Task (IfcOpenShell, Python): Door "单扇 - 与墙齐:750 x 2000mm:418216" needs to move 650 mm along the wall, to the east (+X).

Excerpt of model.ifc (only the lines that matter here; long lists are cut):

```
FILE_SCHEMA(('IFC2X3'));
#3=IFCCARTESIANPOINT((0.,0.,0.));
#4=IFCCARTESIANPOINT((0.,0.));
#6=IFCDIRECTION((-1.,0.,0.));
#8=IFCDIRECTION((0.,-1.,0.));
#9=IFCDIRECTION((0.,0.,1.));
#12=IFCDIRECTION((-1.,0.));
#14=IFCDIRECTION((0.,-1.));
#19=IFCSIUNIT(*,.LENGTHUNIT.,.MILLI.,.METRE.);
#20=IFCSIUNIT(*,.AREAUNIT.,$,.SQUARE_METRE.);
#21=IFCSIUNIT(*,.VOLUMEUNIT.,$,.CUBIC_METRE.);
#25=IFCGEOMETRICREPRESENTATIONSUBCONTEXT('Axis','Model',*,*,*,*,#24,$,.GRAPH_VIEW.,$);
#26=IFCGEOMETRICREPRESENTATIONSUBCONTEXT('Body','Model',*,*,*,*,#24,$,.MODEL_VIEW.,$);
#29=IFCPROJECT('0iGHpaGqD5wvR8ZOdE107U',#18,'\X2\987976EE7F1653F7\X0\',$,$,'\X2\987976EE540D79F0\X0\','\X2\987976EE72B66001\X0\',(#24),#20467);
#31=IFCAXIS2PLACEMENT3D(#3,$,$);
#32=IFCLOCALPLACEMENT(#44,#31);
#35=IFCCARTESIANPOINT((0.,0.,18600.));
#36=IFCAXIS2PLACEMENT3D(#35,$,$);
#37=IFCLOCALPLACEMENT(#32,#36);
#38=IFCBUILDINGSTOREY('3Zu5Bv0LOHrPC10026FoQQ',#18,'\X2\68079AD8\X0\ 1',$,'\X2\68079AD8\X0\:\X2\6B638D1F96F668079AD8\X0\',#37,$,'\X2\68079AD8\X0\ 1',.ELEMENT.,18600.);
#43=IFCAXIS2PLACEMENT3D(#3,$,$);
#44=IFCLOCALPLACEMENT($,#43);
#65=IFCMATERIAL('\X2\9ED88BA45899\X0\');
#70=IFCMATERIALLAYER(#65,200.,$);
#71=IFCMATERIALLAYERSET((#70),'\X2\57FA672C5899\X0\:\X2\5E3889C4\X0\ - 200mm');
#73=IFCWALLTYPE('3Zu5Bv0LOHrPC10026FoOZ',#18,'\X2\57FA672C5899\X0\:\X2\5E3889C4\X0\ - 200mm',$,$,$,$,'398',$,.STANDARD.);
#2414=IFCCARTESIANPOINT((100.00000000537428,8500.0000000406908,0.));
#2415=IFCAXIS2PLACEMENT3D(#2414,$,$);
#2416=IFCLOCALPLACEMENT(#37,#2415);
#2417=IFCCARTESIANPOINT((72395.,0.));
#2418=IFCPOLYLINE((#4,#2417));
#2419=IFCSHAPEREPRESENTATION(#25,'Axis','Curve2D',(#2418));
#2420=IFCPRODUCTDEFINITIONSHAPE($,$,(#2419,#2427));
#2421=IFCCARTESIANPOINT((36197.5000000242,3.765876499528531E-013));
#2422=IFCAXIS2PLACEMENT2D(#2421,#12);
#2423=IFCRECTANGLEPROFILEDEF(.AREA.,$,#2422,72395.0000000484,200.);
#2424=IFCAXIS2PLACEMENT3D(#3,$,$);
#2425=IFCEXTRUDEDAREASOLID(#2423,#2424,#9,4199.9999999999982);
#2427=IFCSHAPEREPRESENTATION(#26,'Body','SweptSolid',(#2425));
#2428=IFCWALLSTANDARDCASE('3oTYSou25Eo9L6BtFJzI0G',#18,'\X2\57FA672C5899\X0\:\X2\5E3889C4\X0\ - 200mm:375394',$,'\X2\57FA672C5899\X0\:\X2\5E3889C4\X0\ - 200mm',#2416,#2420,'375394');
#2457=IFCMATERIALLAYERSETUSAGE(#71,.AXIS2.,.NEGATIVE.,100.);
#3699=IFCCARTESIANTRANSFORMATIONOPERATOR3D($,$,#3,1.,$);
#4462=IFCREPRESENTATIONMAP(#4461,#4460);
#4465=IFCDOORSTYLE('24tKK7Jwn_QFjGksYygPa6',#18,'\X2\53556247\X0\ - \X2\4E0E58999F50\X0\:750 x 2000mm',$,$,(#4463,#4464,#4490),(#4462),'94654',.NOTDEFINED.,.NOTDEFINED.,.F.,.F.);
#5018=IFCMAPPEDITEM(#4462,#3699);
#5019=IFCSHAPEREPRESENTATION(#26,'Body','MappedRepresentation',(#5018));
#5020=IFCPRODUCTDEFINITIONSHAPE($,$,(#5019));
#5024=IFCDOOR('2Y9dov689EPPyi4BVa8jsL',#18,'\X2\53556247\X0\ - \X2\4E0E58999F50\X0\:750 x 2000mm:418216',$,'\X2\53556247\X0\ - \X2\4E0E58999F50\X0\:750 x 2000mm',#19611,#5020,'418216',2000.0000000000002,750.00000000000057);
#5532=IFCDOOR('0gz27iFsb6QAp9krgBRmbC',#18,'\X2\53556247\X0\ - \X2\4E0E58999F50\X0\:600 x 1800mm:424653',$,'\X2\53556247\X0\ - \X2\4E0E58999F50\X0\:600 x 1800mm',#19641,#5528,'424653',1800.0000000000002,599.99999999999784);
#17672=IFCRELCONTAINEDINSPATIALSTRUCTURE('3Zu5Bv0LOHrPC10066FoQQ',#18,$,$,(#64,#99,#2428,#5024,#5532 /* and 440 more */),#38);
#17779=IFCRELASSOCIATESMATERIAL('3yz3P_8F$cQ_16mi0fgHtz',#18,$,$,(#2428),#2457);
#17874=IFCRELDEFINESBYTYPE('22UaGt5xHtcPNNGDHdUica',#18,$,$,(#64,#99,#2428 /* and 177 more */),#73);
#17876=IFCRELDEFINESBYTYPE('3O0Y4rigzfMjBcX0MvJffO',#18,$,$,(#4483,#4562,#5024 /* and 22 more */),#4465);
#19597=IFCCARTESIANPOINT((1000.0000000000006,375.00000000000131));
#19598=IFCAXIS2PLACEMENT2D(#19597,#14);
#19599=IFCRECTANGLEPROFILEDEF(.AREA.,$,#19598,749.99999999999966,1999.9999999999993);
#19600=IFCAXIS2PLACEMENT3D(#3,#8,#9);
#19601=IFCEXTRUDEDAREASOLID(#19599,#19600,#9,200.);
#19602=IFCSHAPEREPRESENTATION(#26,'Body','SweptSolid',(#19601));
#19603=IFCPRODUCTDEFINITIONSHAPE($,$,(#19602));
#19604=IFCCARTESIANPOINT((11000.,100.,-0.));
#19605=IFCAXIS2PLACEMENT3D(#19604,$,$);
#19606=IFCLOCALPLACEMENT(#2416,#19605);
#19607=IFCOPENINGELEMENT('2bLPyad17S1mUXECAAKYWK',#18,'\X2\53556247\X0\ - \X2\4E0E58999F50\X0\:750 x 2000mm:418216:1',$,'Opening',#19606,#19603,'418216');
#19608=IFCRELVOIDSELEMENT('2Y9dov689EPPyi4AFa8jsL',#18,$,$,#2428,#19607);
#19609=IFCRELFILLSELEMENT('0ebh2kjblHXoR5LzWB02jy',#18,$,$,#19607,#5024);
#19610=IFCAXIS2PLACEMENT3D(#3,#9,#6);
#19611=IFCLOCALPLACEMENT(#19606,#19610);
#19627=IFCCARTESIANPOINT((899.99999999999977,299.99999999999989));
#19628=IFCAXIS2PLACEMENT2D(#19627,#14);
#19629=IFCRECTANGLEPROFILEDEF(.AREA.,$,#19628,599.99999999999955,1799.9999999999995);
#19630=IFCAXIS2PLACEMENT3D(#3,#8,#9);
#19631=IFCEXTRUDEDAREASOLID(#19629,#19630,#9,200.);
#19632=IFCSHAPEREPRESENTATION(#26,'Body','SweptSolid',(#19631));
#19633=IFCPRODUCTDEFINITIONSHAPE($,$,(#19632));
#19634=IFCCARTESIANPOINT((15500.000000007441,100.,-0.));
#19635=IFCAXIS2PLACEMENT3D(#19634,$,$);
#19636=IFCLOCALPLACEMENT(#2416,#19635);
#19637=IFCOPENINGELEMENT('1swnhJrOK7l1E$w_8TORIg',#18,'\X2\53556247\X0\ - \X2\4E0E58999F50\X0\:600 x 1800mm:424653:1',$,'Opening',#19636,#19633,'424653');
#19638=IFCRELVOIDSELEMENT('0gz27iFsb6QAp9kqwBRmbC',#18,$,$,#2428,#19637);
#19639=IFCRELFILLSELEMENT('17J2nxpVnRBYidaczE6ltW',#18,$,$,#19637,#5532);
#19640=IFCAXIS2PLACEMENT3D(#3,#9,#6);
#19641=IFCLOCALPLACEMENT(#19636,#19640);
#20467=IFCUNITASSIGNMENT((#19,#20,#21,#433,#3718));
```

```python
import ifcopenshell
import ifcopenshell.api.geometry
import ifcopenshell.util.placement
import ifcopenshell.util.unit

model = ifcopenshell.open("model.ifc")
unit_scale = ifcopenshell.util.unit.calculate_unit_scale(model)

door = model.by_id(5024)
opening = door.FillsVoids[0].RelatingOpeningElement
wall = opening.VoidsElements[0].RelatingBuildingElement

wall_matrix = ifcopenshell.util.placement.get_local_placement(wall.ObjectPlacement)
shift = wall_matrix[:3, 0] * 0.65 / unit_scale
before = ifcopenshell.util.placement.get_local_placement(door.ObjectPlacement)[:3, 3].copy()

# The door is placed relative to its opening, so it follows when the opening moves.
matrix = ifcopenshell.util.placement.get_local_placement(opening.ObjectPlacement)
matrix[:3, 3] += shift
ifcopenshell.api.geometry.edit_object_placement(
    model, product=opening, matrix=matrix, is_si=False, should_transform_children=True
)

after = ifcopenshell.util.placement.get_local_placement(door.ObjectPlacement)[:3, 3]
print("door moved by", (after - before).round(3) + 0.0)

model.write("model_rev.ifc")
```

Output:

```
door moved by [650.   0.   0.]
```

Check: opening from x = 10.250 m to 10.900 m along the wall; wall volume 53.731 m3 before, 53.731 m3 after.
